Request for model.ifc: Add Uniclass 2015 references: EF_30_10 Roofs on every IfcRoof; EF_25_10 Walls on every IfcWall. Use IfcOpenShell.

First a look at what the model holds.

```python
import ifcopenshell

model = ifcopenshell.open("model.ifc")
print(model.schema)
print("classifications:", [c.Name for c in model.by_type("IfcClassification")])
for ifc_class in ("IfcDoor", "IfcRoof", "IfcStair", "IfcWall", "IfcWindow"):
    print(ifc_class, len(model.by_type(ifc_class)))
```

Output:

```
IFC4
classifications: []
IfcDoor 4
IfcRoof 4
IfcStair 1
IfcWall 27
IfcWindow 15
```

```python
import ifcopenshell
import ifcopenshell.api.classification

model = ifcopenshell.open("model.ifc")

system = ifcopenshell.api.classification.add_classification(model, classification="Uniclass 2015")

codes = {
    "IfcRoof": ("EF_30_10", "Roofs"),
    "IfcWall": ("EF_25_10", "Walls"),
}
for ifc_class, (code, name) in codes.items():
    products = model.by_type(ifc_class)
    ifcopenshell.api.classification.add_reference(
        model, products=products, classification=system, identification=code, name=name
    )
    print(code, len(products))

model.write("model_updated.ifc")
```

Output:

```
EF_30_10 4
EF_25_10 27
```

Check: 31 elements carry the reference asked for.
